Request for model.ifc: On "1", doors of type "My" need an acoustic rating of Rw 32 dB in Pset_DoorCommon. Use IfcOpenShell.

First a look at what the model holds.

```python
import ifcopenshell
import ifcopenshell.util.element

model = ifcopenshell.open("model.ifc")
print(model.schema)
storey = next(s for s in model.by_type("IfcBuildingStorey") if s.Name == "1")
doors = [e for e in ifcopenshell.util.element.get_decomposition(storey) if e.is_a("IfcDoor")]
seen = {}
for e in doors:
    element_type = ifcopenshell.util.element.get_type(e)
    key = (element_type.Name if element_type != e and element_type else None, ifcopenshell.util.element.get_pset(e, "Pset_DoorCommon", "AcousticRating"))
    seen[key] = seen.get(key, 0) + 1
for (name, value), count in sorted(seen.items(), key=str):
    print(count, "x", name, "|", value)
```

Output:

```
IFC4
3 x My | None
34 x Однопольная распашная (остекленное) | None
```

```python
import ifcopenshell
import ifcopenshell.api.pset
import ifcopenshell.util.element

model = ifcopenshell.open("model.ifc")

storey = next(s for s in model.by_type("IfcBuildingStorey") if s.Name == "1")
doors = [e for e in ifcopenshell.util.element.get_decomposition(storey) if e.is_a("IfcDoor")]

count = 0
for e in doors:
    element_type = ifcopenshell.util.element.get_type(e)
    if element_type in (None, e) or element_type.Name != "My":
        continue
    # add_pset returns the element's existing set when there is one.
    pset = ifcopenshell.api.pset.add_pset(model, product=e, name="Pset_DoorCommon")
    ifcopenshell.api.pset.edit_pset(model, pset=pset, properties={"AcousticRating": "Rw 32 dB"})
    count += 1

print(count, "doors updated")

model.write("model_edited.ifc")
```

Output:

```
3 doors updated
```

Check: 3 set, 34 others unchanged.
